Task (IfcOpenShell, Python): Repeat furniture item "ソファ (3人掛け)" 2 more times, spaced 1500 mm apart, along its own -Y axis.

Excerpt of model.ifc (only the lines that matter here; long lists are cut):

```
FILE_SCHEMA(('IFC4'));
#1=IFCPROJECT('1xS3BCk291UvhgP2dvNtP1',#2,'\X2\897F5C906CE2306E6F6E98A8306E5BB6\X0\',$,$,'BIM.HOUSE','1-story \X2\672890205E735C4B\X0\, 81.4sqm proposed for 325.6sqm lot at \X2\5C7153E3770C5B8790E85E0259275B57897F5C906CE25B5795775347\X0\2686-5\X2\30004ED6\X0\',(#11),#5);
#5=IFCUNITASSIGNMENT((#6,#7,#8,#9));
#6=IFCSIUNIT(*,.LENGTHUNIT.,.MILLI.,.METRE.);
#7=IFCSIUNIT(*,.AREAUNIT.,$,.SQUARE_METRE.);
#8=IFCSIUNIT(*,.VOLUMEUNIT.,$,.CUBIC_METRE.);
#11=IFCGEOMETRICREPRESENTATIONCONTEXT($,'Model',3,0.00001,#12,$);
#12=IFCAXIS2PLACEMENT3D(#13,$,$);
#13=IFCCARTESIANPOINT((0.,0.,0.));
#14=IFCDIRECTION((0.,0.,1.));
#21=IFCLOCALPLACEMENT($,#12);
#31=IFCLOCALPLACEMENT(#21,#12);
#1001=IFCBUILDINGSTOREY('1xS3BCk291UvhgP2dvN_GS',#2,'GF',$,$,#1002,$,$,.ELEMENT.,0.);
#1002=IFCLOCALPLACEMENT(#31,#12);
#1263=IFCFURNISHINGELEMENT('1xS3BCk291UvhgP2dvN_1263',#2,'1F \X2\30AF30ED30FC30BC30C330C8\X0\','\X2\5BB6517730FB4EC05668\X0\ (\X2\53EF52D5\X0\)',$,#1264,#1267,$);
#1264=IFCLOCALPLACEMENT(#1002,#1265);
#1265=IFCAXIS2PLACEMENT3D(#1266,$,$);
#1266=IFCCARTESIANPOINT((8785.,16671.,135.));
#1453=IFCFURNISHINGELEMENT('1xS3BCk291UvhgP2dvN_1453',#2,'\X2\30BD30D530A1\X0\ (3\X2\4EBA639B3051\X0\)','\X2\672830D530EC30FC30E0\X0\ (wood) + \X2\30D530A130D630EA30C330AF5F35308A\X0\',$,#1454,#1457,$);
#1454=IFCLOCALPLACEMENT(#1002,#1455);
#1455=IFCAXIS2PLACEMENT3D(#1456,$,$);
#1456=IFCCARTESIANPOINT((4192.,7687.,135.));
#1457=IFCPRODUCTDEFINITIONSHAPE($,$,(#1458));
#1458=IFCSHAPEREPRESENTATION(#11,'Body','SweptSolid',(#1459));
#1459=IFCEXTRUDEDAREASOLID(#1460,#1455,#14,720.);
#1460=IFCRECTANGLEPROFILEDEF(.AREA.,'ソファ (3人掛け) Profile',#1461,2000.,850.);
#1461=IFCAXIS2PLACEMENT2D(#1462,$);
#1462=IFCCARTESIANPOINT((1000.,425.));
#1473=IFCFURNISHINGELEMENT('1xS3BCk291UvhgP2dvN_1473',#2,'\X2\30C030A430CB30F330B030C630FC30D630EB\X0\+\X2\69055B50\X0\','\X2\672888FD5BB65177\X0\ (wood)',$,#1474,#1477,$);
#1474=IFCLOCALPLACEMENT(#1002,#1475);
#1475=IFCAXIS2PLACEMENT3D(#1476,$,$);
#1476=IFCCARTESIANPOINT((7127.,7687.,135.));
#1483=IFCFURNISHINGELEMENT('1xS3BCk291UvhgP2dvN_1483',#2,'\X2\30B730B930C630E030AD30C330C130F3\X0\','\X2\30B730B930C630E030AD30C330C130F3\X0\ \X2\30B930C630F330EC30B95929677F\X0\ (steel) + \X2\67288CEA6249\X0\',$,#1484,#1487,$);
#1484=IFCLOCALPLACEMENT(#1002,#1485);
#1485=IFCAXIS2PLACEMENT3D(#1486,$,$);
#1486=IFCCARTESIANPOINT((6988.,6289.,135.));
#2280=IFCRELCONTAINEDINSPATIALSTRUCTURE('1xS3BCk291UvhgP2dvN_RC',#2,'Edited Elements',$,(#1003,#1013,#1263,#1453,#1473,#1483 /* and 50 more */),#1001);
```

```python
import ifcopenshell
import ifcopenshell.api.geometry
import ifcopenshell.api.root
import ifcopenshell.util.element
import ifcopenshell.util.placement

model = ifcopenshell.open("model.ifc")


def reuse_history(source, copy):
    """copy_class also copies each property set's owner history, people and application; keep the originals."""
    for rel in copy.IsDefinedBy:
        if rel.is_a("IfcRelDefinesByProperties") and (history := rel.RelatingPropertyDefinition.OwnerHistory):
            rel.RelatingPropertyDefinition.OwnerHistory = source.OwnerHistory
            ifcopenshell.util.element.remove_deep2(model, history)


source = model.by_guid("1xS3BCk291UvhgP2dvN_1453")
base = ifcopenshell.util.placement.get_local_placement(source.ObjectPlacement)
step = -base[:3, 1] * 1500.0

for i in range(1, 3):
    copy = ifcopenshell.api.root.copy_class(model, product=source)
    copy.Representation = ifcopenshell.util.element.copy_deep(
        model, source.Representation, exclude=["IfcGeometricRepresentationContext", "IfcRepresentationMap"]
    )
    reuse_history(source, copy)
    matrix = base.copy()
    matrix[:3, 3] += i * step
    print("added at", matrix[:3, 3].round(3) + 0.0)
    ifcopenshell.api.geometry.edit_object_placement(model, product=copy, matrix=matrix, is_si=False)

model.write("model-out.ifc")
```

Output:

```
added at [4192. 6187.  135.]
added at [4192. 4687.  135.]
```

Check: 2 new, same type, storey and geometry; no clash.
